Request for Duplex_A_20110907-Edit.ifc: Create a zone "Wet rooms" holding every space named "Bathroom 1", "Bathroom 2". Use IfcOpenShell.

First a look at what the model holds.

```python
import ifcopenshell

model = ifcopenshell.open("Duplex_A_20110907-Edit.ifc")
print(model.schema)
seen = {}
for space in model.by_type("IfcSpace"):
    seen[space.LongName] = seen.get(space.LongName, 0) + 1
for name, count in sorted(seen.items(), key=str):
    print(count, "x", name)
print("zones:", [z.Name for z in model.by_type("IfcZone")][:20])
```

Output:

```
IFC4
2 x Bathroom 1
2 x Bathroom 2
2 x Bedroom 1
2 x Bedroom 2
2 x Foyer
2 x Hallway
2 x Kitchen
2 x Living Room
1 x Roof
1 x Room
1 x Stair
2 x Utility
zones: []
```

```python
import ifcopenshell
import ifcopenshell.api.group
import ifcopenshell.api.root

model = ifcopenshell.open("Duplex_A_20110907-Edit.ifc")

names = {"Bathroom 1", "Bathroom 2"}
spaces = [s for s in model.by_type("IfcSpace") if s.LongName in names]

zone = ifcopenshell.api.root.create_entity(model, ifc_class="IfcZone", name="Wet rooms")
ifcopenshell.api.group.assign_group(model, products=spaces, group=zone)
print(len(spaces), "spaces in", zone.Name)

model.write("Duplex_A_20110907-Edit-out.ifc")
```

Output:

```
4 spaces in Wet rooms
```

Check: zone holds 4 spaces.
